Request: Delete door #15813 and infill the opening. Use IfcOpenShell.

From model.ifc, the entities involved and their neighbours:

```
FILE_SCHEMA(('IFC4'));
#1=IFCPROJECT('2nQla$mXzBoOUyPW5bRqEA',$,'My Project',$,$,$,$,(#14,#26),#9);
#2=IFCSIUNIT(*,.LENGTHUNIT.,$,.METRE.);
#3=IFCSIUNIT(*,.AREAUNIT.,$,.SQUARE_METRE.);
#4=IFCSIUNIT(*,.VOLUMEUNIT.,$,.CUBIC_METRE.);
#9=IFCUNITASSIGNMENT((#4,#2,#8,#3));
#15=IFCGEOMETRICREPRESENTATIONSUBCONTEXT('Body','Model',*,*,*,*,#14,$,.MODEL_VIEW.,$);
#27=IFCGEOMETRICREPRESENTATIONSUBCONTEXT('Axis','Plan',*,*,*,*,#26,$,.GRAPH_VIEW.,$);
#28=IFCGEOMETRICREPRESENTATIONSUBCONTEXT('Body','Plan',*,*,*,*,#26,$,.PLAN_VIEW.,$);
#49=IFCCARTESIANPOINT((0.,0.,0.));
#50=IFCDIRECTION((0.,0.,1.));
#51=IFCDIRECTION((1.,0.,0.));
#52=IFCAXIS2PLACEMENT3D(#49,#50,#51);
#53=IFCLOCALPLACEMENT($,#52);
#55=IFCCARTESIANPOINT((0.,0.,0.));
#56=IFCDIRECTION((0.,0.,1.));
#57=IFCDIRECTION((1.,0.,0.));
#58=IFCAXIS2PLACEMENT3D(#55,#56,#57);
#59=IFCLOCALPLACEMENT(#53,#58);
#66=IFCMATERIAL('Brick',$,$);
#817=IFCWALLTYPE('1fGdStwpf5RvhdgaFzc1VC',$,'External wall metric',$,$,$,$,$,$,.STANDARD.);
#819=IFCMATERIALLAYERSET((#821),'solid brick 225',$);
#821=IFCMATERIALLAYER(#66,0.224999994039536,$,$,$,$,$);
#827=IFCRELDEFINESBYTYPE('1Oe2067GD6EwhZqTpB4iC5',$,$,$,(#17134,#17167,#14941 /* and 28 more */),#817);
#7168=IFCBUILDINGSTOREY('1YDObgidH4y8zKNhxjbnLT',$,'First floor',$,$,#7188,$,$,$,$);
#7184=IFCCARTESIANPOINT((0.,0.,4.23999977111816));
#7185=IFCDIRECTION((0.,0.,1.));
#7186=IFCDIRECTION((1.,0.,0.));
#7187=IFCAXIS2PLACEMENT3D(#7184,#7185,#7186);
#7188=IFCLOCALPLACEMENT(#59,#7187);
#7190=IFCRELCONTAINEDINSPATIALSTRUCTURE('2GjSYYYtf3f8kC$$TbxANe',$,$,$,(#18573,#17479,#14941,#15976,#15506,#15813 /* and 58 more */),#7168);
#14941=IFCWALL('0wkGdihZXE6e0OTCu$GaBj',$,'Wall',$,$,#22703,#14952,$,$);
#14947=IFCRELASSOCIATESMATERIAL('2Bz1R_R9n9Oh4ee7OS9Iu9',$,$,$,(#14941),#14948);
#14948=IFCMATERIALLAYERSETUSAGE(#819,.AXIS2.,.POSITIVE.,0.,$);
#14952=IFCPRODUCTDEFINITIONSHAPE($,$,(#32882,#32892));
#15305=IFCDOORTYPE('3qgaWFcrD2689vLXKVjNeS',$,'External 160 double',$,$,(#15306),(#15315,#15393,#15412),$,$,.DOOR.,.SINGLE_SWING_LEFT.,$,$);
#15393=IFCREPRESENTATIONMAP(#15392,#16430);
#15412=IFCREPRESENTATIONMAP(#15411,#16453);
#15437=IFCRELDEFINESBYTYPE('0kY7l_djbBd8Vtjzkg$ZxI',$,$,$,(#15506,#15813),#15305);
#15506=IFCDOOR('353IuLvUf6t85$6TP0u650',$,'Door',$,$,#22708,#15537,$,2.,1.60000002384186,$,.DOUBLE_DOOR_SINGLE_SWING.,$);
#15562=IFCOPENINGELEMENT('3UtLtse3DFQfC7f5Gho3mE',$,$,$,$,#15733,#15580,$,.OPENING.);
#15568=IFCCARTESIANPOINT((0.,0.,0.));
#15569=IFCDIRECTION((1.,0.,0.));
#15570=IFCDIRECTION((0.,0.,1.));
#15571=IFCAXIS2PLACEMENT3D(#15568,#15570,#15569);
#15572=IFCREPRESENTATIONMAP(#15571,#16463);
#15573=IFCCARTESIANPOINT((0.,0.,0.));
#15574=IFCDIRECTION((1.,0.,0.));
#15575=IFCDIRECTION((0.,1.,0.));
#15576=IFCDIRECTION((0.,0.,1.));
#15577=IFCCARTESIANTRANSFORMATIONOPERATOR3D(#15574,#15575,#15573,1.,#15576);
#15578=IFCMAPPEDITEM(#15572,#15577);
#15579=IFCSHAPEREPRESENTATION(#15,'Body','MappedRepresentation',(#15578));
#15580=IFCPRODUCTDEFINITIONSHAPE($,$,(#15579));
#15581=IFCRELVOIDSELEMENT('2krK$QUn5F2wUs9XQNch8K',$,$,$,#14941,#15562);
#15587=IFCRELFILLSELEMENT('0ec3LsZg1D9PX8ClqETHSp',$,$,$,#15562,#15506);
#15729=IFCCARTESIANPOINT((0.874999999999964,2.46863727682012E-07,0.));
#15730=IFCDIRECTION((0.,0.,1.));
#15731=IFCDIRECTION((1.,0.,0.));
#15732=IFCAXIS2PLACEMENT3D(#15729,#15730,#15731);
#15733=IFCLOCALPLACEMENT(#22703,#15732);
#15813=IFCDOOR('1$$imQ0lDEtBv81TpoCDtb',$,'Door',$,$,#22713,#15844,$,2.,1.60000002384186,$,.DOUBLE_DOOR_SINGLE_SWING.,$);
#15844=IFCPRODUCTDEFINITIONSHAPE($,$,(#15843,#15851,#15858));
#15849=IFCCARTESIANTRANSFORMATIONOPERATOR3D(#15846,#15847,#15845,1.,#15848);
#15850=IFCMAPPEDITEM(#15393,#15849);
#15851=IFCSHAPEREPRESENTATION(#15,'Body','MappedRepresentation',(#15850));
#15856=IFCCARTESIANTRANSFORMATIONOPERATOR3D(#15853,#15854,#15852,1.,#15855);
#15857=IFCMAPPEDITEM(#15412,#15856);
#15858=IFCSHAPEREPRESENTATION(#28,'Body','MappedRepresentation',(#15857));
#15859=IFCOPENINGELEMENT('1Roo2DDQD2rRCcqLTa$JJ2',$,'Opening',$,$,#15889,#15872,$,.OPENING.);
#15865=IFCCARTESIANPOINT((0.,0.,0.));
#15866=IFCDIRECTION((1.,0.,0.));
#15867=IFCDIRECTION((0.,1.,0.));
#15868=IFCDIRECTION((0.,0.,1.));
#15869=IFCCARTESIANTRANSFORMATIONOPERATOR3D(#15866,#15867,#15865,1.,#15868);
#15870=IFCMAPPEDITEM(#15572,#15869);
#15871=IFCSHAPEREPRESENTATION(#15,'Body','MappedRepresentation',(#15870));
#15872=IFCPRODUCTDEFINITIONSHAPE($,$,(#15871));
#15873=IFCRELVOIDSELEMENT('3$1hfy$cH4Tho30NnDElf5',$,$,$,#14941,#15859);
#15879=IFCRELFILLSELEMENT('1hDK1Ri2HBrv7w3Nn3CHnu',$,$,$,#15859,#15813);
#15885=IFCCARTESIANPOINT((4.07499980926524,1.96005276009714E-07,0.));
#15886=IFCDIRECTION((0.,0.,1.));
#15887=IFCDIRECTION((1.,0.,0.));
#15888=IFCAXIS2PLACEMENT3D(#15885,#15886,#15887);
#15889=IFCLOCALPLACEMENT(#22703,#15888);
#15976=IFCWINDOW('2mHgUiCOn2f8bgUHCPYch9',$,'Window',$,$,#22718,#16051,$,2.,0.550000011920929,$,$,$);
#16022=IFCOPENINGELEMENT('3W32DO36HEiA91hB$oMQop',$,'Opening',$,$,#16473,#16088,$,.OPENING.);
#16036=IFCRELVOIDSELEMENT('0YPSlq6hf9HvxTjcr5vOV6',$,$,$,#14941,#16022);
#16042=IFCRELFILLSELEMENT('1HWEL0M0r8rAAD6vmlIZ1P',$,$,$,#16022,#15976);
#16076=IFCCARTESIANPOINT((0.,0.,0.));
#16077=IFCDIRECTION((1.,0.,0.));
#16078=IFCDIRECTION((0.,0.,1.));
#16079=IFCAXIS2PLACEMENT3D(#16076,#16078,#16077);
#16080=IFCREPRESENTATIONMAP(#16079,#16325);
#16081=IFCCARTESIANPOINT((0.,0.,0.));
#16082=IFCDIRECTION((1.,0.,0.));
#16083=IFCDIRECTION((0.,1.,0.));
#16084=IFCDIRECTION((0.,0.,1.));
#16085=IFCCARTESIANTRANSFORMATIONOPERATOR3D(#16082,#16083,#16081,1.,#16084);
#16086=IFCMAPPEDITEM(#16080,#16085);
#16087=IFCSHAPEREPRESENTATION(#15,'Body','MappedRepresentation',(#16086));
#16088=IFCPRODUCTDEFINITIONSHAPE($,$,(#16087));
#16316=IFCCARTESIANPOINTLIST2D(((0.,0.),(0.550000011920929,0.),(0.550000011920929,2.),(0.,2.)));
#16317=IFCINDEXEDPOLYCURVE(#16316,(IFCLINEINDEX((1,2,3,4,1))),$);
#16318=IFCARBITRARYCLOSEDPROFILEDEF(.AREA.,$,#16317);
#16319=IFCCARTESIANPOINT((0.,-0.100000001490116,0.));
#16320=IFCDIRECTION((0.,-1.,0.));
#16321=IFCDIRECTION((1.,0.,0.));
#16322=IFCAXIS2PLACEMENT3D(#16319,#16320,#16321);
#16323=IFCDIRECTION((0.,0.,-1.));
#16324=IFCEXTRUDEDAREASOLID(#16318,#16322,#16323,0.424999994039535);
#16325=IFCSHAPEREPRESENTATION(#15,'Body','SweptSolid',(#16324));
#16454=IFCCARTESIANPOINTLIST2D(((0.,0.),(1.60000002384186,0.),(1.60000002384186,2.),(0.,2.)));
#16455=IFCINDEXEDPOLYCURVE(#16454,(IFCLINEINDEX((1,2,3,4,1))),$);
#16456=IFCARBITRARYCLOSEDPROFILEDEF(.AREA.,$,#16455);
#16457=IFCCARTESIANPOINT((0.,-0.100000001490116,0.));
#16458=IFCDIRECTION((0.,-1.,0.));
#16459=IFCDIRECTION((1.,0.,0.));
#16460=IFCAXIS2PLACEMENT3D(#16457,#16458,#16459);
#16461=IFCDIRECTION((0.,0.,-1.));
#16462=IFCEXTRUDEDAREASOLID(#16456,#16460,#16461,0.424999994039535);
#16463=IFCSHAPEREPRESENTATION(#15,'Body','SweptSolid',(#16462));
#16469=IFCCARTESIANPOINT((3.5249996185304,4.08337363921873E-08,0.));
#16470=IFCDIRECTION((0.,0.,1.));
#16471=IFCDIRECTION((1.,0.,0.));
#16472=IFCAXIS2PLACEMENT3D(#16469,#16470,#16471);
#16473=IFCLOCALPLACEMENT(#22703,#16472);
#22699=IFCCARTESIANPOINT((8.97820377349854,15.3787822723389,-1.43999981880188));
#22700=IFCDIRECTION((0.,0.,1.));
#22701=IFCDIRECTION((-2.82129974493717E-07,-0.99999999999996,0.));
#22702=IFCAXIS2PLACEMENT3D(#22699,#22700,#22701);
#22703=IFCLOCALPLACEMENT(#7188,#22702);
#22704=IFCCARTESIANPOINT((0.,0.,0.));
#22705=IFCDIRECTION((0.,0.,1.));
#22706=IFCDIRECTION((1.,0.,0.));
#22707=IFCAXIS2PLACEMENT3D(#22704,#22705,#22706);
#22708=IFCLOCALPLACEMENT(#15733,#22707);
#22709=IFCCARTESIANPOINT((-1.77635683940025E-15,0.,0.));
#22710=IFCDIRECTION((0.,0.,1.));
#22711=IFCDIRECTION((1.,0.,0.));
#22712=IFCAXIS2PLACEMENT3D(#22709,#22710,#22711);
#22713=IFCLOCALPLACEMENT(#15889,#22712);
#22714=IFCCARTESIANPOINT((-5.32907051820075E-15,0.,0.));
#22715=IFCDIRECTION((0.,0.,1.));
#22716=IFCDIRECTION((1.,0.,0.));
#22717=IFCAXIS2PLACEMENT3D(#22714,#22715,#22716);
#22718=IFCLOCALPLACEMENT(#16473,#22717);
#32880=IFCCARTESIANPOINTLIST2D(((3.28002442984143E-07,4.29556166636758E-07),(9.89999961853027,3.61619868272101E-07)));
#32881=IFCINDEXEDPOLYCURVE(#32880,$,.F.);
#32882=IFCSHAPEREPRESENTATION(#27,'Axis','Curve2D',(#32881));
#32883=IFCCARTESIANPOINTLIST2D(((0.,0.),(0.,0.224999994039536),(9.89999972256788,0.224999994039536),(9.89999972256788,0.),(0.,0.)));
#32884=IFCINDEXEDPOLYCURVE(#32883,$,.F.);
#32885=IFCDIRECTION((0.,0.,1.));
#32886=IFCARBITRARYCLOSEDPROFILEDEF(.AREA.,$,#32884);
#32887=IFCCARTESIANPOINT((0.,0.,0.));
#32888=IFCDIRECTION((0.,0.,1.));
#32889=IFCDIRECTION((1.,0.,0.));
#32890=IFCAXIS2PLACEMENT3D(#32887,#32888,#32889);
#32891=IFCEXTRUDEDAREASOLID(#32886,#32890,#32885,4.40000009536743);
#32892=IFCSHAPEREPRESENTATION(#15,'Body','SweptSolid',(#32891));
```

```python
import ifcopenshell
import ifcopenshell.api.feature
import ifcopenshell.api.root
import ifcopenshell.geom
import ifcopenshell.util.shape

model = ifcopenshell.open("model.ifc")
settings = ifcopenshell.geom.settings()


def volume(element):
    """Net volume in cubic metres, openings subtracted."""
    shape = ifcopenshell.geom.create_shape(settings, element)
    return ifcopenshell.util.shape.get_volume(shape.geometry)


door = model.by_guid("1$$imQ0lDEtBv81TpoCDtb")
opening = door.FillsVoids[0].RelatingOpeningElement
wall = opening.VoidsElements[0].RelatingBuildingElement
before = volume(wall)

ifcopenshell.api.root.remove_product(model, product=door)
ifcopenshell.api.feature.remove_feature(model, feature=opening)

after = volume(wall)

print(f"wall volume {before:.3f} -> {after:.3f} m3")

model.write("model_updated.ifc")
```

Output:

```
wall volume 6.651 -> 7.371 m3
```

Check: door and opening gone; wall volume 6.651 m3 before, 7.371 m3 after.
